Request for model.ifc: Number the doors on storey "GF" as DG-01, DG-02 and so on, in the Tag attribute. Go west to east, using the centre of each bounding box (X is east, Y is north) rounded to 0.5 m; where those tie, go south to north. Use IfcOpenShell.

First a look at what the model holds.

```python
import ifcopenshell
import ifcopenshell.util.element
import ifcopenshell.util.placement

model = ifcopenshell.open("model.ifc")
print(model.schema)
storey = next(s for s in model.by_type("IfcBuildingStorey") if s.Name == "GF")
doors = [e for e in ifcopenshell.util.element.get_decomposition(storey) if e.is_a("IfcDoor")]
for e in sorted(doors, key=lambda e: e.id()):
    origin = ifcopenshell.util.placement.get_local_placement(e.ObjectPlacement)[:3, 3]
    print(e.id(), e.Tag, e.Name, origin.round(2) + 0.0, sep=" | ")
```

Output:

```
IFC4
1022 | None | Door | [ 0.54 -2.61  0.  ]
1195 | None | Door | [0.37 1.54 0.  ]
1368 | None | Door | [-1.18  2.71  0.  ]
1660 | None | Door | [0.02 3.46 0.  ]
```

```python
import ifcopenshell
import ifcopenshell.geom
import ifcopenshell.util.element
import ifcopenshell.util.shape

model = ifcopenshell.open("model.ifc")
settings = ifcopenshell.geom.settings()
settings.set("use-world-coords", True)


def centre(element):
    shape = ifcopenshell.geom.create_shape(settings, element)
    return ifcopenshell.util.shape.get_bbox_centroid(shape.geometry)


storey = next(s for s in model.by_type("IfcBuildingStorey") if s.Name == "GF")
doors = [e for e in ifcopenshell.util.element.get_decomposition(storey) if e.is_a("IfcDoor")]

# Insertion points can sit at a corner or the storey origin, so sort by the geometry (in metres).
centres = {e: centre(e) for e in doors}
doors.sort(key=lambda e: (round(centres[e][0] / 0.5), centres[e][1]))

for i, e in enumerate(doors, start=1):
    number = f"DG-{i:02d}"
    e.Tag = number
    print(e.id(), number)

model.write("model-out.ifc")
```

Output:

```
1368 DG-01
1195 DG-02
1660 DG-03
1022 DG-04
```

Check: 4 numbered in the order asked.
